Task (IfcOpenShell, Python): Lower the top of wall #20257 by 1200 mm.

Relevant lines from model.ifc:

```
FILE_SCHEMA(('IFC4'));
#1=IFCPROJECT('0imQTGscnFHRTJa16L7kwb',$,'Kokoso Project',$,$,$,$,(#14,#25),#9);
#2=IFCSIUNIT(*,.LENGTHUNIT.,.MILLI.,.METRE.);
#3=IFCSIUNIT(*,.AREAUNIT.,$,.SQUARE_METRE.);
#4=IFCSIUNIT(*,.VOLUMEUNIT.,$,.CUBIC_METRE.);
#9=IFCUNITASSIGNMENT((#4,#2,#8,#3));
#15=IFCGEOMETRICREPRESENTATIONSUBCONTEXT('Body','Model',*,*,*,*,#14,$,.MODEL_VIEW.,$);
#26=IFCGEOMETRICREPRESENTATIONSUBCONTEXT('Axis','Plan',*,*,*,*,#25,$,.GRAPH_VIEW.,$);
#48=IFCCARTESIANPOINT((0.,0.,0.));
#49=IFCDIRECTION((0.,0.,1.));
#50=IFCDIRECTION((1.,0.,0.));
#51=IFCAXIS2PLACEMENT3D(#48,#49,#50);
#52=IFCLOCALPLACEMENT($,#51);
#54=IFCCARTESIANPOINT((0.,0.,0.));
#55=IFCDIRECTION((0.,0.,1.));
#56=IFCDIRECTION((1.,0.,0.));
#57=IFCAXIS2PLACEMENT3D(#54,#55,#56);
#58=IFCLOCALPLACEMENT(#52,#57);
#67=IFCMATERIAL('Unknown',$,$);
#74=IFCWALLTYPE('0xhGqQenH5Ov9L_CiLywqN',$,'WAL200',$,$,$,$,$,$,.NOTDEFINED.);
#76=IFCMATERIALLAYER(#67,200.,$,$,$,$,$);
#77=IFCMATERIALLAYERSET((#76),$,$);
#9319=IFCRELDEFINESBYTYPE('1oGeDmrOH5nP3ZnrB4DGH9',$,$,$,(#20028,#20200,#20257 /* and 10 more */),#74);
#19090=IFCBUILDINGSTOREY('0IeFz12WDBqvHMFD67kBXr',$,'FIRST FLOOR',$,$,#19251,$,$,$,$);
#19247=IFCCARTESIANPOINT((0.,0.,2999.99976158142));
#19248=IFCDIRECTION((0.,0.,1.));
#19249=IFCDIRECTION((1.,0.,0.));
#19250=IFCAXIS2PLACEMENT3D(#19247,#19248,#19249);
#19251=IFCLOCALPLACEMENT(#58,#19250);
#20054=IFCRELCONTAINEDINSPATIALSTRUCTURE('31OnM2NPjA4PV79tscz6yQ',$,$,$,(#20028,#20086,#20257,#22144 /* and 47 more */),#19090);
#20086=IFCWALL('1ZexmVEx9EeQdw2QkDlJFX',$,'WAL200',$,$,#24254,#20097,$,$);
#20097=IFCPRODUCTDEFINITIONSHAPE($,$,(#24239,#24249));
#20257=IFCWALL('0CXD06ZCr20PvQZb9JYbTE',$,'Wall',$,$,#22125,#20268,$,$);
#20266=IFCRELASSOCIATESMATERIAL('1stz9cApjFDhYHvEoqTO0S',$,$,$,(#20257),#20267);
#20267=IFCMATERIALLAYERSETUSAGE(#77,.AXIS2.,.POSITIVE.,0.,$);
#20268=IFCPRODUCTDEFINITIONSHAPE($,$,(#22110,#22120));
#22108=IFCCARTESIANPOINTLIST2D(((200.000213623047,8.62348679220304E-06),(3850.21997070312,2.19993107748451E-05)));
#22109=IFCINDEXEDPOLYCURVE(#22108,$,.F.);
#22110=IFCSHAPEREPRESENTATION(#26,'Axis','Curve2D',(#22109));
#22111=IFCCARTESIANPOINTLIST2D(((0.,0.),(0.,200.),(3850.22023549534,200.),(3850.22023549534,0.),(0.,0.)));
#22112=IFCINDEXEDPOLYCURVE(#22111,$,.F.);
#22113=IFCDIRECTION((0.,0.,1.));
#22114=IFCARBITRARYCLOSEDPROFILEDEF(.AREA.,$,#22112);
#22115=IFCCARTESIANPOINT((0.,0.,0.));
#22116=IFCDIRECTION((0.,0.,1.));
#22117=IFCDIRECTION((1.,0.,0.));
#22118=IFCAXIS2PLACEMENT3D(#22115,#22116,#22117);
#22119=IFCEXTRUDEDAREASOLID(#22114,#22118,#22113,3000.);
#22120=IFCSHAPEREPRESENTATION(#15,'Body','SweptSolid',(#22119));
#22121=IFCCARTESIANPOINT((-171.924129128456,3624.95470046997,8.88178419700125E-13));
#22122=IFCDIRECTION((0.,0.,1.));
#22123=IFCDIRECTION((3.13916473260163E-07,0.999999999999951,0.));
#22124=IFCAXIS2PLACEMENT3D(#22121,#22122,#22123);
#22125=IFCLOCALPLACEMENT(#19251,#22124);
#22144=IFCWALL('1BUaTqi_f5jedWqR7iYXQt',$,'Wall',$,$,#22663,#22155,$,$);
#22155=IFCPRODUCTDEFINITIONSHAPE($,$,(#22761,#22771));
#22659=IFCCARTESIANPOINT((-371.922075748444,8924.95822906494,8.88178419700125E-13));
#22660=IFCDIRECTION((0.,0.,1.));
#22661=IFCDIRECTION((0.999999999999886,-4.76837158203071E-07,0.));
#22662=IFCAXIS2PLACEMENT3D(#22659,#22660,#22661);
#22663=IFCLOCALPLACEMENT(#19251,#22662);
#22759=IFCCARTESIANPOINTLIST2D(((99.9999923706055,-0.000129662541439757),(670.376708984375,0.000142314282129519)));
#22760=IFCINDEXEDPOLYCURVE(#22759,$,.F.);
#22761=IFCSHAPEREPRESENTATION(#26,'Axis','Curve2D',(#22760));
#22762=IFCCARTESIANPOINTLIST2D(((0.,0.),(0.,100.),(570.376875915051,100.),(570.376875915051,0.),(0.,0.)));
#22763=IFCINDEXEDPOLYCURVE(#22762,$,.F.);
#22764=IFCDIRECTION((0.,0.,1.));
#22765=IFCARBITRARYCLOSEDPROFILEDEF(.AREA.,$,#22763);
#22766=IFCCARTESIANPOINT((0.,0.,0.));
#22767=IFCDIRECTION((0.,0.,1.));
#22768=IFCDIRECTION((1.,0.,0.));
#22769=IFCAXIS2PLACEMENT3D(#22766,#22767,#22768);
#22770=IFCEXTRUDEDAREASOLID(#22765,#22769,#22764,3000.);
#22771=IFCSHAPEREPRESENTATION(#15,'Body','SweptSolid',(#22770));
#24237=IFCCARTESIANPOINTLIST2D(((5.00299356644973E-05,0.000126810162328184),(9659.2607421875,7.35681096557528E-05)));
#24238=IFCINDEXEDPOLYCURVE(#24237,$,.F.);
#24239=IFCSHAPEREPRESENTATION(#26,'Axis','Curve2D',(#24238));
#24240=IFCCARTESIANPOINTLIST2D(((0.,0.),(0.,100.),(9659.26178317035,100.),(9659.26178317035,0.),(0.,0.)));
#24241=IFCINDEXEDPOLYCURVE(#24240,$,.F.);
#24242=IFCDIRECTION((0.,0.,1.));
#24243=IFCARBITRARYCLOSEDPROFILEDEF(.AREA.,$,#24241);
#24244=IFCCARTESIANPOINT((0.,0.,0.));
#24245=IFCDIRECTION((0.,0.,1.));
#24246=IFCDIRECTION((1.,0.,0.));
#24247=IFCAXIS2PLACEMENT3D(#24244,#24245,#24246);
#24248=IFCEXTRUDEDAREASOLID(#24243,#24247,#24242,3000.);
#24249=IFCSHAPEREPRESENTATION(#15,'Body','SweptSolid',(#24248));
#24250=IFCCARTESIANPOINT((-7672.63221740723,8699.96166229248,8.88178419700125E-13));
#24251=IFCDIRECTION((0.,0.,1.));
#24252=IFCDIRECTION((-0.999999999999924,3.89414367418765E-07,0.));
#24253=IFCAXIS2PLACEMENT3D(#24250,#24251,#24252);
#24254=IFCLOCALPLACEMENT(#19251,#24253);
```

```python
import ifcopenshell
import ifcopenshell.geom
import ifcopenshell.util.representation
import ifcopenshell.util.shape
import ifcopenshell.util.unit

model = ifcopenshell.open("model.ifc")
unit_scale = ifcopenshell.util.unit.calculate_unit_scale(model)
settings = ifcopenshell.geom.settings()


def volume(element):
    """Net volume in cubic metres, openings subtracted."""
    shape = ifcopenshell.geom.create_shape(settings, element)
    return ifcopenshell.util.shape.get_volume(shape.geometry)


wall = model.by_id(20257)
before = volume(wall)

body = ifcopenshell.util.representation.get_representation(wall, "Model", "Body")
solid = body.Items[0]
old_height = solid.Depth
solid.Depth -= 1.2 / unit_scale
after = volume(wall)

print(f"height {old_height:g} -> {solid.Depth:g}, volume {before:.3f} -> {after:.3f} m3")

model.write("model_updated.ifc")
```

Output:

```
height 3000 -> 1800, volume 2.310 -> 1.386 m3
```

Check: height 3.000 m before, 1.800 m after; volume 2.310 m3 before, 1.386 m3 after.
